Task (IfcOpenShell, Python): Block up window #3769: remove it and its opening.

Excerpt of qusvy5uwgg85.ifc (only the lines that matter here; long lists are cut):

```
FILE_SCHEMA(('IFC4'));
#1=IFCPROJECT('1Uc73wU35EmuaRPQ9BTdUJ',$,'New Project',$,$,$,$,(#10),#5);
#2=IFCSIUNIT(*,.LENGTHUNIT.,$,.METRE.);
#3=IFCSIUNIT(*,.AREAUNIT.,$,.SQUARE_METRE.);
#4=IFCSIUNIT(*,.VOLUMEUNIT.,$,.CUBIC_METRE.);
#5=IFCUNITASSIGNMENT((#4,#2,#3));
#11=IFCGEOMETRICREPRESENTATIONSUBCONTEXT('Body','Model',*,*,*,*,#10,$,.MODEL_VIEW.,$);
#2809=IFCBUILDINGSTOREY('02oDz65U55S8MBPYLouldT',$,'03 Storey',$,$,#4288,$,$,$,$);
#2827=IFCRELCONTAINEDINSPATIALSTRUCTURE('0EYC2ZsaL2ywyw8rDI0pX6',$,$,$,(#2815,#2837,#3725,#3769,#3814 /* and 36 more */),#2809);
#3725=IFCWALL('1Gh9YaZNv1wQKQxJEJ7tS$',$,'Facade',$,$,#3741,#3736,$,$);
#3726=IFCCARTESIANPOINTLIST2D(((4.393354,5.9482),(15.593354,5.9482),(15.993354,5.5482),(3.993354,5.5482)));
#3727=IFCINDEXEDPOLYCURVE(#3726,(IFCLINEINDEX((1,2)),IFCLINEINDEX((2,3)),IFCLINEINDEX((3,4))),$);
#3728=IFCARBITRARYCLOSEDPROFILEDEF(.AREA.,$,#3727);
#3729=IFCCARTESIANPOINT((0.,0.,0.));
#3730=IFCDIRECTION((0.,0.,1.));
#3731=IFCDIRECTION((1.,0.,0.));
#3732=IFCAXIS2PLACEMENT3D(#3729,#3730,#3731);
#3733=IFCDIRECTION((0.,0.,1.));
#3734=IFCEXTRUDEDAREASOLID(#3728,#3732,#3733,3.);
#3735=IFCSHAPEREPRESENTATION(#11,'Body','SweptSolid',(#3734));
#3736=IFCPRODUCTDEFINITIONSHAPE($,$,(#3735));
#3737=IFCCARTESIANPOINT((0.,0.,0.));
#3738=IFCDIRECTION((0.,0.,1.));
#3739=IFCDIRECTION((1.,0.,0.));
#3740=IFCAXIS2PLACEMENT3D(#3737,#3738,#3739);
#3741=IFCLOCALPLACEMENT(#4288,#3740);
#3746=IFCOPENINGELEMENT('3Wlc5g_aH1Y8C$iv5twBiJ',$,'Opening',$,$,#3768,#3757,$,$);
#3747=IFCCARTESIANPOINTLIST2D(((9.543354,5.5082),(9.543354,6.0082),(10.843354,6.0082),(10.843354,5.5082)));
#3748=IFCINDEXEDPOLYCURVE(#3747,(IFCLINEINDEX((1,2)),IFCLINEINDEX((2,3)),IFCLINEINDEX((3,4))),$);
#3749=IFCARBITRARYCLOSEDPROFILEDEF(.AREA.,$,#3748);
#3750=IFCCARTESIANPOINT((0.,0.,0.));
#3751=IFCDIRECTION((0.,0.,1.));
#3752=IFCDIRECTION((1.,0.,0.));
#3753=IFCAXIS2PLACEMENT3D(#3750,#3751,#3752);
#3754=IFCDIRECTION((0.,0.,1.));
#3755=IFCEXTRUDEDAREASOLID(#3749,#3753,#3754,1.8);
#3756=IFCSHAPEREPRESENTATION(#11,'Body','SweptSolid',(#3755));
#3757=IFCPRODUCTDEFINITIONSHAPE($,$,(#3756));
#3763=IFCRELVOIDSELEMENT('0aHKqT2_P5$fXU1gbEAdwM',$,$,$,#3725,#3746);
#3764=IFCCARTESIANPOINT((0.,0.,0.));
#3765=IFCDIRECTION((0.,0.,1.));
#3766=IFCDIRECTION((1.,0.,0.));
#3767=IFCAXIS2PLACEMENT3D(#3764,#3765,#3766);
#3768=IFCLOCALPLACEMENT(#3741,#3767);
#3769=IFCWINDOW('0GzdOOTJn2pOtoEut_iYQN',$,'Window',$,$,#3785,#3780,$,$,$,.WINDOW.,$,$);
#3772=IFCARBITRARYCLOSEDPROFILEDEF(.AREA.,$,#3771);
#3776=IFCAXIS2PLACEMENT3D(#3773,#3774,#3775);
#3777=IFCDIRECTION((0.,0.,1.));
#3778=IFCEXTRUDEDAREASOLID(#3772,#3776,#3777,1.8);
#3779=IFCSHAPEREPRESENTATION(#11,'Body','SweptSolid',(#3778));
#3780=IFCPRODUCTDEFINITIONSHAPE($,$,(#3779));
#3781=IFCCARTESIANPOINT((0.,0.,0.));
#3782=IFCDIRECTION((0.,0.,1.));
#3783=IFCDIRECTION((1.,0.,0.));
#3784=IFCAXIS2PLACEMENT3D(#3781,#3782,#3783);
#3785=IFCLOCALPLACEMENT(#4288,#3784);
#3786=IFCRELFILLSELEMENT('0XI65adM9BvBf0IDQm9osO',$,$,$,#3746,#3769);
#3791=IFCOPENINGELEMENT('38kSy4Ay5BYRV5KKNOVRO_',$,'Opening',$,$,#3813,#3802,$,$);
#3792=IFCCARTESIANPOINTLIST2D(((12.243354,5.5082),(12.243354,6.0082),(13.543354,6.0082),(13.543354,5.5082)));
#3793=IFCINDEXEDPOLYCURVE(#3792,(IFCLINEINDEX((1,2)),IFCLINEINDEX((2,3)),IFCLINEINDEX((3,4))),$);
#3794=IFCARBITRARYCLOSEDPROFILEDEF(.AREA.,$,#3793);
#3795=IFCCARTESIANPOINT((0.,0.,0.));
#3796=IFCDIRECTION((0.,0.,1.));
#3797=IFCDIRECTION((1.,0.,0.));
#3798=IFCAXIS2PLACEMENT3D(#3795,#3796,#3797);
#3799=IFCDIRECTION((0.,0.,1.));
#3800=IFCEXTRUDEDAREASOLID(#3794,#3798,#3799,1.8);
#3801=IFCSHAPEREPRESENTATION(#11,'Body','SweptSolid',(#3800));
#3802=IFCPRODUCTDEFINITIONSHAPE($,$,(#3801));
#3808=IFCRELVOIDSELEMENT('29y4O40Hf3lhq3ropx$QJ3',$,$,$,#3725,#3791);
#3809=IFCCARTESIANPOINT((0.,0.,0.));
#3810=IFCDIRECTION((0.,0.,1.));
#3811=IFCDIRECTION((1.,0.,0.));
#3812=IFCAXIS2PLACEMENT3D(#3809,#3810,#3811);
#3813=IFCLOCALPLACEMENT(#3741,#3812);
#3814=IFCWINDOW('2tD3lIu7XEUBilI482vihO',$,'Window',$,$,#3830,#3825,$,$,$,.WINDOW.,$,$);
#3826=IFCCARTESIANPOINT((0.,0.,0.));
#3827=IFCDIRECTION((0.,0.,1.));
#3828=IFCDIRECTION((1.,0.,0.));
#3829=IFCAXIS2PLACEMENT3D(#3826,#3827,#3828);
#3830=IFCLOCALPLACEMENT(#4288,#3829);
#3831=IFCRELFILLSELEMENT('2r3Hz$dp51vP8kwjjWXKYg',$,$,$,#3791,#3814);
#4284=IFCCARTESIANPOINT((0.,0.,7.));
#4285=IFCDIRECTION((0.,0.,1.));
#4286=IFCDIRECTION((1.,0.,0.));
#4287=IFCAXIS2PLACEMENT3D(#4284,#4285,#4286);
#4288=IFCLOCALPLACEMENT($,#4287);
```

```python
import ifcopenshell
import ifcopenshell.api.feature
import ifcopenshell.api.root
import ifcopenshell.geom
import ifcopenshell.util.shape

model = ifcopenshell.open("qusvy5uwgg85.ifc")
settings = ifcopenshell.geom.settings()


def volume(element):
    """Net volume in cubic metres, openings subtracted."""
    shape = ifcopenshell.geom.create_shape(settings, element)
    return ifcopenshell.util.shape.get_volume(shape.geometry)


window = model.by_id(3769)
opening = window.FillsVoids[0].RelatingOpeningElement
wall = opening.VoidsElements[0].RelatingBuildingElement
before = volume(wall)

ifcopenshell.api.root.remove_product(model, product=window)
ifcopenshell.api.feature.remove_feature(model, feature=opening)

after = volume(wall)

print(f"wall volume {before:.3f} -> {after:.3f} m3")

model.write("qusvy5uwgg85_edited.ifc")
```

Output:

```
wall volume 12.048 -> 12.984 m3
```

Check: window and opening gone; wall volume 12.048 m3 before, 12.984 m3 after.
